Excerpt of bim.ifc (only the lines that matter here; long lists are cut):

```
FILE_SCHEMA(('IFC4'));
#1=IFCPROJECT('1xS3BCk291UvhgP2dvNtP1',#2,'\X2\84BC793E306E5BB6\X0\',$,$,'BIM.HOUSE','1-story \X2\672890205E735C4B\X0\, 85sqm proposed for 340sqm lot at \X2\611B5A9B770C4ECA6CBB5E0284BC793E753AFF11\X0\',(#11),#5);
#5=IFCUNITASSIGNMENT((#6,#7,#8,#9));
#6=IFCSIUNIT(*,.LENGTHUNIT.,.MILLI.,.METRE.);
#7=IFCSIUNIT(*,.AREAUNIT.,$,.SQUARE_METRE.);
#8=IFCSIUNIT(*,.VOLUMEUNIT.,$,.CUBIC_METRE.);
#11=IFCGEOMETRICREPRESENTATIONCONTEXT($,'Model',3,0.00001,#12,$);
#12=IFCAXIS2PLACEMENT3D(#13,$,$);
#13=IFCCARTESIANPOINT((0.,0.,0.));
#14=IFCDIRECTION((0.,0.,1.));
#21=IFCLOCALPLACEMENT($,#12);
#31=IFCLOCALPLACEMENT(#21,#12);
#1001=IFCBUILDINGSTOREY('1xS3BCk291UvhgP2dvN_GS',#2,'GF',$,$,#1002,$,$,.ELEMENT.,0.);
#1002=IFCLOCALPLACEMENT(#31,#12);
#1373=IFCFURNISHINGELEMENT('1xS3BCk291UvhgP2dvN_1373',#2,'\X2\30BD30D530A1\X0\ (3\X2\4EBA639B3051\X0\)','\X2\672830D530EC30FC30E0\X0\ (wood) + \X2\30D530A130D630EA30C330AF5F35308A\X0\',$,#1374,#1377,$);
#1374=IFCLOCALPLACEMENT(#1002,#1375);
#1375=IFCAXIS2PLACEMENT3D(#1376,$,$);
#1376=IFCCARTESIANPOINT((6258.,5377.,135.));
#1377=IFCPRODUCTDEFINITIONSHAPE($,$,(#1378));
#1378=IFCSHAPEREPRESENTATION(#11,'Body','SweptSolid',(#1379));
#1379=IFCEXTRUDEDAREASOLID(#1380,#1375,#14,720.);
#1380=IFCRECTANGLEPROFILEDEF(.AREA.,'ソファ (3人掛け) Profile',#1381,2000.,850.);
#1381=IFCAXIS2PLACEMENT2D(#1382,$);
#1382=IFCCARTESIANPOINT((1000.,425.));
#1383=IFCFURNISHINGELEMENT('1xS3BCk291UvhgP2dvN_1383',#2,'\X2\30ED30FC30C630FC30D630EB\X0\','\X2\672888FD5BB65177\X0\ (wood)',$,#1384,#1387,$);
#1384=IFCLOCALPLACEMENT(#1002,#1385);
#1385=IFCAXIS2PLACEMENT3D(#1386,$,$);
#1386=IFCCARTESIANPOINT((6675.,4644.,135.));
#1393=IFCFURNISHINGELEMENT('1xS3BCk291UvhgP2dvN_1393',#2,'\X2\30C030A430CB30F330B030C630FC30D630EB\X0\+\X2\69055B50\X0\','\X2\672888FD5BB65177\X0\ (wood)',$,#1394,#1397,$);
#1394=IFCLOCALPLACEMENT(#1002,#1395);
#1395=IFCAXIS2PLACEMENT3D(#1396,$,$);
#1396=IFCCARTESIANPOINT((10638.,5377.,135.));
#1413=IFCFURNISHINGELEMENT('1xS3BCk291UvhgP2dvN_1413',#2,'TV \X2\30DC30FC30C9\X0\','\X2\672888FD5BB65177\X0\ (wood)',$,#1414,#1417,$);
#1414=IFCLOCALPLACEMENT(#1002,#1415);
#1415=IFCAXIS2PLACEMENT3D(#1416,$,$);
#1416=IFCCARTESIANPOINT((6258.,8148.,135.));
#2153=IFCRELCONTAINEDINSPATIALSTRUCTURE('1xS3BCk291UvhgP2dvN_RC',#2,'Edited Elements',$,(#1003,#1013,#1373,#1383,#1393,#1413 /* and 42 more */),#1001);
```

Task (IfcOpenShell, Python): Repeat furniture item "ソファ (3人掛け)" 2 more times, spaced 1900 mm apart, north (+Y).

```python
import numpy as np
import ifcopenshell
import ifcopenshell.api.geometry
import ifcopenshell.api.root
import ifcopenshell.util.element
import ifcopenshell.util.placement

model = ifcopenshell.open("bim.ifc")


def reuse_history(source, copy):
    """copy_class also copies each property set's owner history, people and application; keep the originals."""
    for rel in copy.IsDefinedBy:
        if rel.is_a("IfcRelDefinesByProperties") and (history := rel.RelatingPropertyDefinition.OwnerHistory):
            rel.RelatingPropertyDefinition.OwnerHistory = source.OwnerHistory
            ifcopenshell.util.element.remove_deep2(model, history)


source = model.by_id(1373)
base = ifcopenshell.util.placement.get_local_placement(source.ObjectPlacement)
step = np.array([0.0, 1.0, 0.0]) * 1900.0

for i in range(1, 3):
    copy = ifcopenshell.api.root.copy_class(model, product=source)
    copy.Representation = ifcopenshell.util.element.copy_deep(
        model, source.Representation, exclude=["IfcGeometricRepresentationContext", "IfcRepresentationMap"]
    )
    reuse_history(source, copy)
    matrix = base.copy()
    matrix[:3, 3] += i * step
    print("added at", matrix[:3, 3].round(3) + 0.0)
    ifcopenshell.api.geometry.edit_object_placement(model, product=copy, matrix=matrix, is_si=False)

model.write("bim_edited.ifc")
```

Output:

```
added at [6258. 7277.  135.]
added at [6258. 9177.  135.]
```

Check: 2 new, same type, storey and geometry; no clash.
